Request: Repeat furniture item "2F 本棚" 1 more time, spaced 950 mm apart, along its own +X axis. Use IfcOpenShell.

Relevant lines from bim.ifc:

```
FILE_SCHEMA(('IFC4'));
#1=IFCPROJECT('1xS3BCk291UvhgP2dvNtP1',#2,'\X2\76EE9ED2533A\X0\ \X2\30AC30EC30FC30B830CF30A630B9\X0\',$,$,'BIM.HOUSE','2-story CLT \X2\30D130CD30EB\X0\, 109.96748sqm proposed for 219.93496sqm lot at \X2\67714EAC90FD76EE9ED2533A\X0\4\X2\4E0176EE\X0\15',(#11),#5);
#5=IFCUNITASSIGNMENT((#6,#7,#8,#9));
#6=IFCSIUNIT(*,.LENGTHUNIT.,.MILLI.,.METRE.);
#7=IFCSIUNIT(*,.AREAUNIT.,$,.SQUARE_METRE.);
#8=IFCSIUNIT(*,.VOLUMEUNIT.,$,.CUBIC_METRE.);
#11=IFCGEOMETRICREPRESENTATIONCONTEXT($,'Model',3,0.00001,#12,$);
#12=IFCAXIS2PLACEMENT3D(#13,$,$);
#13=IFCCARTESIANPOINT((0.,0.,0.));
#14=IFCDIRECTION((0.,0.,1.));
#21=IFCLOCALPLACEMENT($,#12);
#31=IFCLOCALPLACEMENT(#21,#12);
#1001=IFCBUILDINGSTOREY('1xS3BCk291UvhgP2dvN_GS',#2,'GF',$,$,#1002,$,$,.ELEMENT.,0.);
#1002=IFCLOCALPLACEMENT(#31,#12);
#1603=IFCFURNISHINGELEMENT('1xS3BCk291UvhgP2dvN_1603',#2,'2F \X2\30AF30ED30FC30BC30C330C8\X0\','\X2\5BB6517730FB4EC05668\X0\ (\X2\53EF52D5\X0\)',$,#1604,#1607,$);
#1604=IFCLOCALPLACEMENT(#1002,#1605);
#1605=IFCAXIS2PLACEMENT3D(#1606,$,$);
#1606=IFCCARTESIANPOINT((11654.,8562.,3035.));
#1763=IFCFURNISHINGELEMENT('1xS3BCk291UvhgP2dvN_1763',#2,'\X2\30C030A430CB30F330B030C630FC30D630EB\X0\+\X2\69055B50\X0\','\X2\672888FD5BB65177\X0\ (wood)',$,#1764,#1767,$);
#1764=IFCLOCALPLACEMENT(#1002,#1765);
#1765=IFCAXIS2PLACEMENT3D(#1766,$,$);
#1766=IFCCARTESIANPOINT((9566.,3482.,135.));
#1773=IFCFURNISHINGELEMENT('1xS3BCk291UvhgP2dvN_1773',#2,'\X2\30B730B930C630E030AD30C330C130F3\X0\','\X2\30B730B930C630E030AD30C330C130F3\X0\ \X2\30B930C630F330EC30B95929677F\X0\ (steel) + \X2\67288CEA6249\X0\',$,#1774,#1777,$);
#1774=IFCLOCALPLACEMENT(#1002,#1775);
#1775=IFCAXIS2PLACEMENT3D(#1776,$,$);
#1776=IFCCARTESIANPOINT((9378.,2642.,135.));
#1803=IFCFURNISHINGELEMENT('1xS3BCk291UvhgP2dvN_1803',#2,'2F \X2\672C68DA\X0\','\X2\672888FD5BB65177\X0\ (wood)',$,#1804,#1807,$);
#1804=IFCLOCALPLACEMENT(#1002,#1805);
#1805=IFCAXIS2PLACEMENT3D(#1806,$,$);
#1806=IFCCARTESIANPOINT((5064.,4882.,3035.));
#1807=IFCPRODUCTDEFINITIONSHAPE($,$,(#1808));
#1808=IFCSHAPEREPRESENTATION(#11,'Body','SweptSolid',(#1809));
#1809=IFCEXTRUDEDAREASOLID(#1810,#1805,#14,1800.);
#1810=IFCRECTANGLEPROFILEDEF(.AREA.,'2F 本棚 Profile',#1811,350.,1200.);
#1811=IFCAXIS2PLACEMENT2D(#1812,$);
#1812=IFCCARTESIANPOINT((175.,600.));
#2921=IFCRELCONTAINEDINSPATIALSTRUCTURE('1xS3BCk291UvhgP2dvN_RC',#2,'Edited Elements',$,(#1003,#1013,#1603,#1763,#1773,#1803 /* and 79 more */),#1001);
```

```python
import ifcopenshell
import ifcopenshell.api.geometry
import ifcopenshell.api.root
import ifcopenshell.util.element
import ifcopenshell.util.placement
import ifcopenshell.util.unit

model = ifcopenshell.open("bim.ifc")
unit_scale = ifcopenshell.util.unit.calculate_unit_scale(model)


def reuse_history(source, copy):
    """copy_class also copies each property set's owner history, people and application; keep the originals."""
    for rel in copy.IsDefinedBy:
        if rel.is_a("IfcRelDefinesByProperties") and (history := rel.RelatingPropertyDefinition.OwnerHistory):
            rel.RelatingPropertyDefinition.OwnerHistory = source.OwnerHistory
            ifcopenshell.util.element.remove_deep2(model, history)


source = model.by_guid("1xS3BCk291UvhgP2dvN_1803")
base = ifcopenshell.util.placement.get_local_placement(source.ObjectPlacement)
step = base[:3, 0] * 0.95 / unit_scale

for i in range(1, 2):
    copy = ifcopenshell.api.root.copy_class(model, product=source)
    copy.Representation = ifcopenshell.util.element.copy_deep(
        model, source.Representation, exclude=["IfcGeometricRepresentationContext", "IfcRepresentationMap"]
    )
    reuse_history(source, copy)
    matrix = base.copy()
    matrix[:3, 3] += i * step
    print("added at", matrix[:3, 3].round(3) + 0.0)
    ifcopenshell.api.geometry.edit_object_placement(model, product=copy, matrix=matrix, is_si=False)

model.write("bim_updated.ifc")
```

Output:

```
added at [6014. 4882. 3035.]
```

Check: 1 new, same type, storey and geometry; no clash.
